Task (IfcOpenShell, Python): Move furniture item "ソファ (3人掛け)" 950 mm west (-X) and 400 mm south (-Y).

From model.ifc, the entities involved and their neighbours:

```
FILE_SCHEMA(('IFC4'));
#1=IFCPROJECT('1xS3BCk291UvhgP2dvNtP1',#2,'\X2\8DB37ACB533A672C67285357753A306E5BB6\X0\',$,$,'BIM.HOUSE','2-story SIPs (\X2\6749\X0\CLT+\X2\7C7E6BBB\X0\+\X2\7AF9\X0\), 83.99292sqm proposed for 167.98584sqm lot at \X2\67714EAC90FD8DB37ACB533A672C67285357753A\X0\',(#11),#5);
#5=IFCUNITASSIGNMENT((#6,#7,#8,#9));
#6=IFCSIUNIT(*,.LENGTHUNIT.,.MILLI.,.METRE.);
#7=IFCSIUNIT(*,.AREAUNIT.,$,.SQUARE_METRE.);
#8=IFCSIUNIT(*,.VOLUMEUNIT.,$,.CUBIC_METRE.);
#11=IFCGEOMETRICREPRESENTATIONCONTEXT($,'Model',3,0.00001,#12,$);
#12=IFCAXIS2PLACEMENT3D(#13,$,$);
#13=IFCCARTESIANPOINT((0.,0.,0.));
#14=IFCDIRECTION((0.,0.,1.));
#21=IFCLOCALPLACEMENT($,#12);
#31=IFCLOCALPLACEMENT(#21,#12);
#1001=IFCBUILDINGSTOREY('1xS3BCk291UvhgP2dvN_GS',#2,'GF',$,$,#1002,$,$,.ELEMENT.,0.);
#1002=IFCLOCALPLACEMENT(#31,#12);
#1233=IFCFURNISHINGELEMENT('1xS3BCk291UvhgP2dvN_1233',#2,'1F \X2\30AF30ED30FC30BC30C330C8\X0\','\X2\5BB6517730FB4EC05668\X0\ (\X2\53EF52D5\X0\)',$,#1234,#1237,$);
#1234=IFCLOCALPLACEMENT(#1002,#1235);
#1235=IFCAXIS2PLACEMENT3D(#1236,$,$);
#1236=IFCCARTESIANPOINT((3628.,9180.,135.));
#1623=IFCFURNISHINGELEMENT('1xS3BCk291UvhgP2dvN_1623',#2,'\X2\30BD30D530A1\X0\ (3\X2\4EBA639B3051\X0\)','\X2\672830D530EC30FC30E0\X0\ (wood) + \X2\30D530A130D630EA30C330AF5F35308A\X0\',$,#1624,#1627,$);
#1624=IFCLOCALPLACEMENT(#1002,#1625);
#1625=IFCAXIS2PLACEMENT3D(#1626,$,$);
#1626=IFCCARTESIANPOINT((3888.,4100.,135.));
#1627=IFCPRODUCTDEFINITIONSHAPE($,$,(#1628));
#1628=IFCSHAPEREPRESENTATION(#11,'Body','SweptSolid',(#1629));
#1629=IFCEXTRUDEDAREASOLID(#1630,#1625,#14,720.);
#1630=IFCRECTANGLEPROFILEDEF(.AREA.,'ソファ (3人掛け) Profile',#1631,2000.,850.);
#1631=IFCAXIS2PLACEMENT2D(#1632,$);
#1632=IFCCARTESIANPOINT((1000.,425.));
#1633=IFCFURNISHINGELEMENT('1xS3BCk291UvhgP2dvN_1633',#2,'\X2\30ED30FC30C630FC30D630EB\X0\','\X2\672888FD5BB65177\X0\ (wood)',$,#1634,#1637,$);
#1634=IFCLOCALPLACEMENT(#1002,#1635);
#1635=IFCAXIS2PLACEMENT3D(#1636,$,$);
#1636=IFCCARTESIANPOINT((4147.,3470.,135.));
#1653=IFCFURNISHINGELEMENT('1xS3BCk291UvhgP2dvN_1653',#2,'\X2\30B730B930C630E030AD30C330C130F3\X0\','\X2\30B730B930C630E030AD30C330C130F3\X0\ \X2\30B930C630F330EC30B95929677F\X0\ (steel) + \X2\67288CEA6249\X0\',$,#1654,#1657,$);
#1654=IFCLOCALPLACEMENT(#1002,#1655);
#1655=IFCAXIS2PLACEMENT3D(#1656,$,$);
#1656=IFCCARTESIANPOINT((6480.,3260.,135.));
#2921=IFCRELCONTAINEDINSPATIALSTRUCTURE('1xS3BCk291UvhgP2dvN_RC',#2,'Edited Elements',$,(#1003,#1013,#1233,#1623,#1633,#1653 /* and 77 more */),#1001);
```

```python
import ifcopenshell
import ifcopenshell.api.geometry
import ifcopenshell.util.placement

model = ifcopenshell.open("model.ifc")

item = model.by_guid("1xS3BCk291UvhgP2dvN_1623")
matrix = ifcopenshell.util.placement.get_local_placement(item.ObjectPlacement)
matrix[0, 3] -= 950.0
matrix[1, 3] -= 400.0
ifcopenshell.api.geometry.edit_object_placement(model, product=item, matrix=matrix, is_si=False)

print(ifcopenshell.util.placement.get_local_placement(item.ObjectPlacement).round(3) + 0.0)

model.write("model_edited.ifc")
```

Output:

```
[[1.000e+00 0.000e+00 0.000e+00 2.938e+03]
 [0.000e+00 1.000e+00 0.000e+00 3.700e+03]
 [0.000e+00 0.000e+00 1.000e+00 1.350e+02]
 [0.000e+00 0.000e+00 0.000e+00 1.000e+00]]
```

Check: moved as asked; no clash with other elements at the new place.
